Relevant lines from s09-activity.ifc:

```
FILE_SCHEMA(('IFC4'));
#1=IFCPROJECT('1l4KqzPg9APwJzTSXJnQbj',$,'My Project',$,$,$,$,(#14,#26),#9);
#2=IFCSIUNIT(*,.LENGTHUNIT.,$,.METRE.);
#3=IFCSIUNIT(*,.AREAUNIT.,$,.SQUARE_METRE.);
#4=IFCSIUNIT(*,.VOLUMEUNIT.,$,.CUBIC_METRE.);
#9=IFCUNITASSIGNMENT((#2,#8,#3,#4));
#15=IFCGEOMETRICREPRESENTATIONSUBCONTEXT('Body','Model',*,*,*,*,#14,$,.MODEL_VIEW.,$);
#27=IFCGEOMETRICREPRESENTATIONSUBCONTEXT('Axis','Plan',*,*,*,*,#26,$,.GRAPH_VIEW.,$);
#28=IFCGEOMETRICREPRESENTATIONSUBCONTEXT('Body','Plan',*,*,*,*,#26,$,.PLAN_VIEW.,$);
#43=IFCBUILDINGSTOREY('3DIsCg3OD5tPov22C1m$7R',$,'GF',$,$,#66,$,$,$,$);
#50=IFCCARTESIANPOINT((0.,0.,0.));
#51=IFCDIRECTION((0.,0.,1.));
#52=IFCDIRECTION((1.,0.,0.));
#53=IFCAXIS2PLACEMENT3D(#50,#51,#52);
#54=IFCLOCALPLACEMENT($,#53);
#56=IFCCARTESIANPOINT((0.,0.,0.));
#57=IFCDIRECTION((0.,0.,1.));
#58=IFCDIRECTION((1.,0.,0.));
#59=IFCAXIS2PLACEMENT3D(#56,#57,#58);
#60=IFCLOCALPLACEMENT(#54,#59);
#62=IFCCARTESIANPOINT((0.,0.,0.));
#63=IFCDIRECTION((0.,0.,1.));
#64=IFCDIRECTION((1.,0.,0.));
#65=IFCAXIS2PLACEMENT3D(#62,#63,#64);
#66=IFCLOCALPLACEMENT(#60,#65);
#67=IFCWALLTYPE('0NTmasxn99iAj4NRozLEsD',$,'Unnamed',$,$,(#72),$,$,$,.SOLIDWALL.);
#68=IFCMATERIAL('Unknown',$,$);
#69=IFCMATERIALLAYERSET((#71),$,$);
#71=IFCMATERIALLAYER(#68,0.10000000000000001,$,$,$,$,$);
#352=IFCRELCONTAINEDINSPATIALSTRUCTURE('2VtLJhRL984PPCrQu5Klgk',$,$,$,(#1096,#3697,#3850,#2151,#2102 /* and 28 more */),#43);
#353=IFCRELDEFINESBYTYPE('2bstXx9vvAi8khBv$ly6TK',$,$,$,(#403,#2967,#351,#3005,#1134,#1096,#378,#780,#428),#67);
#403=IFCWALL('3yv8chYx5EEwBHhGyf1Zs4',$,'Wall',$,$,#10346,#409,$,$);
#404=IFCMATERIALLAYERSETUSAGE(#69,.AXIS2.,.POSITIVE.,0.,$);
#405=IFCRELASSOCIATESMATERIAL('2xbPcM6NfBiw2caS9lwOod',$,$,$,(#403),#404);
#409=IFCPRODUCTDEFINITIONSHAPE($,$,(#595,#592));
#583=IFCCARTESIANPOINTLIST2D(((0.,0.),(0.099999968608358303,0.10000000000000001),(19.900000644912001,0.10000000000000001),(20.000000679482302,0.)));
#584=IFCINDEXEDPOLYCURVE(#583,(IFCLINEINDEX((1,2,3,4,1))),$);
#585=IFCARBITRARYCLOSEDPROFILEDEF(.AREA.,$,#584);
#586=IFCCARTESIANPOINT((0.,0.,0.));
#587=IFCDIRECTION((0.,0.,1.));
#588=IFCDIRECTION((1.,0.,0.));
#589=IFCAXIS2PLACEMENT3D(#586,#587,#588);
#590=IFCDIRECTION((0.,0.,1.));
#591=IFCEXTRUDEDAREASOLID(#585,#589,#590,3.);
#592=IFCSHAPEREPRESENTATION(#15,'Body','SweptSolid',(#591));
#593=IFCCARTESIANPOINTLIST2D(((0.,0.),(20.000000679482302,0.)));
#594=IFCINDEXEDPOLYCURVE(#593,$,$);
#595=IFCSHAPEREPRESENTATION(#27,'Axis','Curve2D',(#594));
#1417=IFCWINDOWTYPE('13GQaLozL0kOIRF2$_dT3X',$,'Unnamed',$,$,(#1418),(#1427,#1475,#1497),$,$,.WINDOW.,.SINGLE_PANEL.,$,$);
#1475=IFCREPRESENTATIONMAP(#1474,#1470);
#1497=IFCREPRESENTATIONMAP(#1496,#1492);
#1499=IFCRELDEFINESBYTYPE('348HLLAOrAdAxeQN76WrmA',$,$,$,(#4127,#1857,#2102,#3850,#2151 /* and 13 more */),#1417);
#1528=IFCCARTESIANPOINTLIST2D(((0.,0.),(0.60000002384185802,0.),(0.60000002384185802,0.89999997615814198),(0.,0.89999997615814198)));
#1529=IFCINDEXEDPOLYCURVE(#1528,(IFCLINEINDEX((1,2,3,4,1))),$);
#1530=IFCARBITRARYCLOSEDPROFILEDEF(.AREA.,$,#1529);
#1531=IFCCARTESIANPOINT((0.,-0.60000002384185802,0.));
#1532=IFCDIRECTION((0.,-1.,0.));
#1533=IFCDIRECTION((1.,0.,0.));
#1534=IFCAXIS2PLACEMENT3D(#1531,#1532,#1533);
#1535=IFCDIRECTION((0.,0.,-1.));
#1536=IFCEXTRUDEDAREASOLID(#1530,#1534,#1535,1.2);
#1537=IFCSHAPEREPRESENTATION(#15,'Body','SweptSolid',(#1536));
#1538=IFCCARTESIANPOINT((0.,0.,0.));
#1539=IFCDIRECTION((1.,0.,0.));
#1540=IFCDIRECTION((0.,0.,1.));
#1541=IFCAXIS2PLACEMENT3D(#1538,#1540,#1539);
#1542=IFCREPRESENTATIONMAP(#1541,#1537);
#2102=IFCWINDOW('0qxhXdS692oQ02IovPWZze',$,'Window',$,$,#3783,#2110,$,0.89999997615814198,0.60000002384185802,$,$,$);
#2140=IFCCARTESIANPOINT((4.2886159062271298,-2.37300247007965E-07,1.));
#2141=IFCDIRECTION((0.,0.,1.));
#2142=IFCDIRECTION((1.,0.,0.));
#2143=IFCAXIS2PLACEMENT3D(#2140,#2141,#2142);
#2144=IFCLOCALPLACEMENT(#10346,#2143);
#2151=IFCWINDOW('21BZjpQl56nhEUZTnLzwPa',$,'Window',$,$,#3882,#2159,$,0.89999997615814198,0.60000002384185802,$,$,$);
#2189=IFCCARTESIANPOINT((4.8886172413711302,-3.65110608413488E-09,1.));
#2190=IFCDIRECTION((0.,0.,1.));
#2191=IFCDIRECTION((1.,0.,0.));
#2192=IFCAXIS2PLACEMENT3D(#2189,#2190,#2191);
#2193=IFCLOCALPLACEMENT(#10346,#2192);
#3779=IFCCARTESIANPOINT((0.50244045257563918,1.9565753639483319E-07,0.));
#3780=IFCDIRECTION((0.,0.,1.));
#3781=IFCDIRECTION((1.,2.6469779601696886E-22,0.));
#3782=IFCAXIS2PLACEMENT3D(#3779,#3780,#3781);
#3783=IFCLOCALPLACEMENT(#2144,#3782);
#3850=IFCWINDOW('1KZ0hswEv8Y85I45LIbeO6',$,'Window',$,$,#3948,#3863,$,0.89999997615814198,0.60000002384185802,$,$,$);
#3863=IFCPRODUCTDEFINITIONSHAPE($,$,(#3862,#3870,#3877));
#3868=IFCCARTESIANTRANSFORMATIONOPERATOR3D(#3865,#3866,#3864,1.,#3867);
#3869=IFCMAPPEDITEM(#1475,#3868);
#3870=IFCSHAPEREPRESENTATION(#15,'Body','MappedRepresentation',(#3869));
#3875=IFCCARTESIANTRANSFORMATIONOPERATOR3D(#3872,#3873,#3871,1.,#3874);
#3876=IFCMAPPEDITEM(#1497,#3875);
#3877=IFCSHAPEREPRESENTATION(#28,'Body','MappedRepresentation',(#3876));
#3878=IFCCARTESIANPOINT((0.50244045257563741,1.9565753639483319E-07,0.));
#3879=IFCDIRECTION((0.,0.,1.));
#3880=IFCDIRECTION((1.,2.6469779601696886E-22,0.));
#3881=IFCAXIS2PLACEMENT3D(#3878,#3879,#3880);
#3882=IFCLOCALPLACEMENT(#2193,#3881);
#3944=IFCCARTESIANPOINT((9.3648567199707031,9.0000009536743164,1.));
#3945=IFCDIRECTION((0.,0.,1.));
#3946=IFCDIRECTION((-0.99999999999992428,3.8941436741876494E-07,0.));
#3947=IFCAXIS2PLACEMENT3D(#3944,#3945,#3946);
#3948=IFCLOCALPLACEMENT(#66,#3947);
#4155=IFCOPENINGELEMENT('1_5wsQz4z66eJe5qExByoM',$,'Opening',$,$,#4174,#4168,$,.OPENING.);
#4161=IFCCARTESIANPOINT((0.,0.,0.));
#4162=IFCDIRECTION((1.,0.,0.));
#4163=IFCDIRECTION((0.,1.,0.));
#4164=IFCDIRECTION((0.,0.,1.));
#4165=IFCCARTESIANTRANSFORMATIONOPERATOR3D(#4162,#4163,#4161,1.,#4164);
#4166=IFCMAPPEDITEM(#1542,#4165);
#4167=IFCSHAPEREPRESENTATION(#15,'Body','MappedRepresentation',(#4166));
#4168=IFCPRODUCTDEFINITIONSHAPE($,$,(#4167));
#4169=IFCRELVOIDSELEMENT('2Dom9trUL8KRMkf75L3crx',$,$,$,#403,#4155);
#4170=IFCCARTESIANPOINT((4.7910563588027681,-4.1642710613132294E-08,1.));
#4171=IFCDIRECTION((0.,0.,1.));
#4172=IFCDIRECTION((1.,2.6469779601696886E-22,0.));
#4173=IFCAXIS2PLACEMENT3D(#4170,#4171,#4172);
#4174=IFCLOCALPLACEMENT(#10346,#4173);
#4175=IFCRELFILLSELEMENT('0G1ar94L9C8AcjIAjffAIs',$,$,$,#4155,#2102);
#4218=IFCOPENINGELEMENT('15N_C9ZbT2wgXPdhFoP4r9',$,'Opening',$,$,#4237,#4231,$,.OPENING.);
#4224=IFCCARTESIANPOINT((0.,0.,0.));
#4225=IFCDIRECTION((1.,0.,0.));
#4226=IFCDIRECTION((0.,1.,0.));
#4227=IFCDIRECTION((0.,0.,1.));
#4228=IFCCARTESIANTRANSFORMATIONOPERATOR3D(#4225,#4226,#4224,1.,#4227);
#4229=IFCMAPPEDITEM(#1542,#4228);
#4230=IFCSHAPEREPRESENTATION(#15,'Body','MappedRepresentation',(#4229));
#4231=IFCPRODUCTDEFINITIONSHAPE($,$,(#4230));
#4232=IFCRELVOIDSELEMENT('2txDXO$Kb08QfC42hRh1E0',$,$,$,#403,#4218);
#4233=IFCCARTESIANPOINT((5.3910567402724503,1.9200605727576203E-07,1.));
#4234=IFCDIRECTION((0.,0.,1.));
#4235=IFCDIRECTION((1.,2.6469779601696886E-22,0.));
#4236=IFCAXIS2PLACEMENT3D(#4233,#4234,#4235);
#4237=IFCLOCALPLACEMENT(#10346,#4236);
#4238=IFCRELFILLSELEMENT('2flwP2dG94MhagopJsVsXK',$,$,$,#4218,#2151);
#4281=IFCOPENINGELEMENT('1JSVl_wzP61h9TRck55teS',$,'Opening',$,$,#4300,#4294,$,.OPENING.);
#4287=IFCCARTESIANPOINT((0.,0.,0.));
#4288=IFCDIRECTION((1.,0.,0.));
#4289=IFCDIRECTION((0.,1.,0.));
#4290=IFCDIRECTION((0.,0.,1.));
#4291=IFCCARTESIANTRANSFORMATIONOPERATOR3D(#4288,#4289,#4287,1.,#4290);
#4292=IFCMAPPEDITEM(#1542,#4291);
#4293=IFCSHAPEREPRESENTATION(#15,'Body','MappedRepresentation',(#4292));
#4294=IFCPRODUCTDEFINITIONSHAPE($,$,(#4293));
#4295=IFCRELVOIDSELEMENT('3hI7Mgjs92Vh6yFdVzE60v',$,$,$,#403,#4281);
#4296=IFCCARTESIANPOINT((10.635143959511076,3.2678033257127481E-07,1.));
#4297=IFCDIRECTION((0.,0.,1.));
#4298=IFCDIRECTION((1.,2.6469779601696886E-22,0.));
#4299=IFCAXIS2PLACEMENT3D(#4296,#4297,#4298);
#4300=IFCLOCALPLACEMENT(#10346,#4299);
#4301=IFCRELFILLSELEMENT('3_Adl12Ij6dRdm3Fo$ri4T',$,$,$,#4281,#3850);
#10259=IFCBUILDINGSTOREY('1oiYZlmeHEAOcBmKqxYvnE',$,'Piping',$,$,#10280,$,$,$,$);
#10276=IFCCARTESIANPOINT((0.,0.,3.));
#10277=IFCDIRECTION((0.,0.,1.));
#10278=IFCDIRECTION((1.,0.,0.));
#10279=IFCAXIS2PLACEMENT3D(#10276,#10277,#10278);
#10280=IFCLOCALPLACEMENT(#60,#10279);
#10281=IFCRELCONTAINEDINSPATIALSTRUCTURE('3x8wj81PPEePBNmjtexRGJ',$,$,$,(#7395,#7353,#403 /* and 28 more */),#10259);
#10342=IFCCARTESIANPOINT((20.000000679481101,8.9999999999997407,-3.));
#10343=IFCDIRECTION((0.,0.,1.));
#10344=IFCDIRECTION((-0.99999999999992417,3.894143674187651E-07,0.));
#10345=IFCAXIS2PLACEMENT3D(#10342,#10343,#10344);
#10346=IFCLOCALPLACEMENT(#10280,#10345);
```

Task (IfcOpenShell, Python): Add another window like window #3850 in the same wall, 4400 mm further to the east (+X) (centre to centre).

```python
import ifcopenshell
import ifcopenshell.api.feature
import ifcopenshell.api.geometry
import ifcopenshell.api.root
import ifcopenshell.geom
import ifcopenshell.util.element
import ifcopenshell.util.placement
import ifcopenshell.util.shape

model = ifcopenshell.open("s09-activity.ifc")
settings = ifcopenshell.geom.settings()


def volume(element):
    """Net volume in cubic metres, openings subtracted."""
    shape = ifcopenshell.geom.create_shape(settings, element)
    return ifcopenshell.util.shape.get_volume(shape.geometry)


window = model.by_id(3850)
opening = window.FillsVoids[0].RelatingOpeningElement
wall = opening.VoidsElements[0].RelatingBuildingElement
before = volume(wall)
shift = ifcopenshell.util.placement.get_local_placement(wall.ObjectPlacement)[:3, 0] * -4.4

# copy_class copies the void relationship, type, container and properties, but no geometry.
new_opening = ifcopenshell.api.root.copy_class(model, product=opening)
new_opening.Representation = ifcopenshell.util.element.copy_deep(
    model, opening.Representation, exclude=["IfcGeometricRepresentationContext", "IfcRepresentationMap"]
)
new_window = ifcopenshell.api.root.copy_class(model, product=window)
new_window.Representation = ifcopenshell.util.element.copy_deep(
    model, window.Representation, exclude=["IfcGeometricRepresentationContext", "IfcRepresentationMap"]
)
ifcopenshell.api.feature.add_filling(model, opening=new_opening, element=new_window)

for old, new in ((opening, new_opening), (window, new_window)):
    matrix = ifcopenshell.util.placement.get_local_placement(old.ObjectPlacement)
    matrix[:3, 3] += shift
    ifcopenshell.api.geometry.edit_object_placement(model, product=new, matrix=matrix, is_si=False)

after = volume(wall)

print(f"wall volume {before:.3f} -> {after:.3f} m3")

model.write("s09-activity_rev.ifc")
```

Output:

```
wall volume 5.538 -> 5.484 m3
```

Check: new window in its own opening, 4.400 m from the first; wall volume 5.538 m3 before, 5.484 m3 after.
